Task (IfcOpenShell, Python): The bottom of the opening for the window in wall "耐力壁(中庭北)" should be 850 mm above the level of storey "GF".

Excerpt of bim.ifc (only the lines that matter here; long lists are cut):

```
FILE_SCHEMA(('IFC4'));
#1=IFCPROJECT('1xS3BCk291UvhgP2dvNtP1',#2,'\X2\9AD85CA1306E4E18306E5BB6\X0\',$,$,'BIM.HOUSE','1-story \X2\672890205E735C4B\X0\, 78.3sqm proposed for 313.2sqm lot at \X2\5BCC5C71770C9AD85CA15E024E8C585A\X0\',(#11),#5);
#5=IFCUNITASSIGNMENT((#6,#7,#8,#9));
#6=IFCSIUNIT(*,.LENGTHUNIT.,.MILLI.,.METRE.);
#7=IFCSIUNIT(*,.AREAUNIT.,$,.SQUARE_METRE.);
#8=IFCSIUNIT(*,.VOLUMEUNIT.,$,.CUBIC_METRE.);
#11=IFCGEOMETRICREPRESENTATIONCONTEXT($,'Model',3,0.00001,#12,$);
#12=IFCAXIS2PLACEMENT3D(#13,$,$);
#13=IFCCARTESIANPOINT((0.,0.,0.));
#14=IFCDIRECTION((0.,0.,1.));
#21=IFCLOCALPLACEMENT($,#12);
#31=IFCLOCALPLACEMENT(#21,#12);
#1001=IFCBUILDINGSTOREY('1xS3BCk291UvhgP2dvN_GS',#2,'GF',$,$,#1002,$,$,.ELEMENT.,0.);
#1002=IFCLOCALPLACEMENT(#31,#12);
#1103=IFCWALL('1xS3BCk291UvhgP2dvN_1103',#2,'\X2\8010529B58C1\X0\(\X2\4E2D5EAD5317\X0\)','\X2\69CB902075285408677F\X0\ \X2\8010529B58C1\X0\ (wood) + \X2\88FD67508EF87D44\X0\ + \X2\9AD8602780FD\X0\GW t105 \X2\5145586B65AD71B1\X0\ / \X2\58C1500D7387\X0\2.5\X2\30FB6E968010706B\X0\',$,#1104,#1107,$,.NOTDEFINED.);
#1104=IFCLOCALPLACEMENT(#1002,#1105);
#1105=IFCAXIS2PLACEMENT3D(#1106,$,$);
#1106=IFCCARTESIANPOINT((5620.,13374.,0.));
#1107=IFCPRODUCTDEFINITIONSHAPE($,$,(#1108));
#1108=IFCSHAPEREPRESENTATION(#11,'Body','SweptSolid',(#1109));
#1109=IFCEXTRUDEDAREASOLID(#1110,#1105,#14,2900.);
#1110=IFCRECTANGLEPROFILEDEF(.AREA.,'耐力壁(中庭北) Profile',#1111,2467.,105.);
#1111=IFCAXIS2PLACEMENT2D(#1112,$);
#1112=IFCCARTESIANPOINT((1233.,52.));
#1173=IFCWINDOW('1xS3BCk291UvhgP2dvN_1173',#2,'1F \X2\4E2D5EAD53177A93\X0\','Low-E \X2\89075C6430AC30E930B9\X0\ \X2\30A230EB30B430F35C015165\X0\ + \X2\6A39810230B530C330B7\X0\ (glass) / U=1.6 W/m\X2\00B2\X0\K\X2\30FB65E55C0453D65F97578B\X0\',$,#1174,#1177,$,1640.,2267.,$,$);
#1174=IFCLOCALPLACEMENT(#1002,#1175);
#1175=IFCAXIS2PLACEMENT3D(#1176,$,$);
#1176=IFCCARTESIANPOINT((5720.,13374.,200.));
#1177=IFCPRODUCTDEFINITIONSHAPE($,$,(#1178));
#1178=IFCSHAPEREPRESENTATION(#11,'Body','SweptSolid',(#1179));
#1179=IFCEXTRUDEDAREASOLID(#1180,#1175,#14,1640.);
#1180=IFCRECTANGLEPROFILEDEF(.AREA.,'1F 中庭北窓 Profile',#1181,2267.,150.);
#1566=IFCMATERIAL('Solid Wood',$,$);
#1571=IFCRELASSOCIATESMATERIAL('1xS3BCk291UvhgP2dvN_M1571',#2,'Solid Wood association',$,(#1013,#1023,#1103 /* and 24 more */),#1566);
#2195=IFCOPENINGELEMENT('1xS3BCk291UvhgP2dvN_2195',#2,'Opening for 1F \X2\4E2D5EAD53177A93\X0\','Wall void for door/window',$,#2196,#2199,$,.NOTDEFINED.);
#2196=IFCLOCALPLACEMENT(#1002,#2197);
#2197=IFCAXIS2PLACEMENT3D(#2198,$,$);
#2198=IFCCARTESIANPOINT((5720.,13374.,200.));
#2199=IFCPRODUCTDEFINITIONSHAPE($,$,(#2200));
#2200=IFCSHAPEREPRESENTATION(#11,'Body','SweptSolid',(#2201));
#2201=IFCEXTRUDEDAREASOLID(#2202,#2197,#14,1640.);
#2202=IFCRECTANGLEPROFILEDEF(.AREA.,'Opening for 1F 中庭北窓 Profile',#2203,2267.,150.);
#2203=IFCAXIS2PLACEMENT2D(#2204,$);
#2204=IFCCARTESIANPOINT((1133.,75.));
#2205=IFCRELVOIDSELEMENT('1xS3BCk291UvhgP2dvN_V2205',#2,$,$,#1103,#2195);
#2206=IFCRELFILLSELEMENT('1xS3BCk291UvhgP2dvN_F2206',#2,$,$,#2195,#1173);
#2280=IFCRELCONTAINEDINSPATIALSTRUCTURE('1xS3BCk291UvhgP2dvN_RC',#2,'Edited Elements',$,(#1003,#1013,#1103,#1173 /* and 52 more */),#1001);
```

```python
import numpy as np
import ifcopenshell
import ifcopenshell.api.geometry
import ifcopenshell.geom
import ifcopenshell.util.element
import ifcopenshell.util.placement
import ifcopenshell.util.shape
import ifcopenshell.util.unit

model = ifcopenshell.open("bim.ifc")
unit_scale = ifcopenshell.util.unit.calculate_unit_scale(model)

window = model.by_id(1173)
opening = window.FillsVoids[0].RelatingOpeningElement
storey = ifcopenshell.util.element.get_container(window, ifc_class="IfcBuildingStorey")
level = ifcopenshell.util.placement.get_local_placement(storey.ObjectPlacement)[2, 3]

# The opening's origin need not be at the sill, so measure its lowest point.
shape = ifcopenshell.geom.create_shape(ifcopenshell.geom.settings(), opening)
bottom = ifcopenshell.util.shape.get_shape_bottom_elevation(shape, shape.geometry) / unit_scale
dz = level + 850.0 - bottom

shift = np.array([0.0, 0.0, dz])
# The window is not placed relative to its opening, so move both.
for product in (opening, window):
    matrix = ifcopenshell.util.placement.get_local_placement(product.ObjectPlacement)
    matrix[:3, 3] += shift
    ifcopenshell.api.geometry.edit_object_placement(model, product=product, matrix=matrix, is_si=False)

print(f"moved by {dz * unit_scale:+.3f} m")

model.write("bim-out.ifc")
```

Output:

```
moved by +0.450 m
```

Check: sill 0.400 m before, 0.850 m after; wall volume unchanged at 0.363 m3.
